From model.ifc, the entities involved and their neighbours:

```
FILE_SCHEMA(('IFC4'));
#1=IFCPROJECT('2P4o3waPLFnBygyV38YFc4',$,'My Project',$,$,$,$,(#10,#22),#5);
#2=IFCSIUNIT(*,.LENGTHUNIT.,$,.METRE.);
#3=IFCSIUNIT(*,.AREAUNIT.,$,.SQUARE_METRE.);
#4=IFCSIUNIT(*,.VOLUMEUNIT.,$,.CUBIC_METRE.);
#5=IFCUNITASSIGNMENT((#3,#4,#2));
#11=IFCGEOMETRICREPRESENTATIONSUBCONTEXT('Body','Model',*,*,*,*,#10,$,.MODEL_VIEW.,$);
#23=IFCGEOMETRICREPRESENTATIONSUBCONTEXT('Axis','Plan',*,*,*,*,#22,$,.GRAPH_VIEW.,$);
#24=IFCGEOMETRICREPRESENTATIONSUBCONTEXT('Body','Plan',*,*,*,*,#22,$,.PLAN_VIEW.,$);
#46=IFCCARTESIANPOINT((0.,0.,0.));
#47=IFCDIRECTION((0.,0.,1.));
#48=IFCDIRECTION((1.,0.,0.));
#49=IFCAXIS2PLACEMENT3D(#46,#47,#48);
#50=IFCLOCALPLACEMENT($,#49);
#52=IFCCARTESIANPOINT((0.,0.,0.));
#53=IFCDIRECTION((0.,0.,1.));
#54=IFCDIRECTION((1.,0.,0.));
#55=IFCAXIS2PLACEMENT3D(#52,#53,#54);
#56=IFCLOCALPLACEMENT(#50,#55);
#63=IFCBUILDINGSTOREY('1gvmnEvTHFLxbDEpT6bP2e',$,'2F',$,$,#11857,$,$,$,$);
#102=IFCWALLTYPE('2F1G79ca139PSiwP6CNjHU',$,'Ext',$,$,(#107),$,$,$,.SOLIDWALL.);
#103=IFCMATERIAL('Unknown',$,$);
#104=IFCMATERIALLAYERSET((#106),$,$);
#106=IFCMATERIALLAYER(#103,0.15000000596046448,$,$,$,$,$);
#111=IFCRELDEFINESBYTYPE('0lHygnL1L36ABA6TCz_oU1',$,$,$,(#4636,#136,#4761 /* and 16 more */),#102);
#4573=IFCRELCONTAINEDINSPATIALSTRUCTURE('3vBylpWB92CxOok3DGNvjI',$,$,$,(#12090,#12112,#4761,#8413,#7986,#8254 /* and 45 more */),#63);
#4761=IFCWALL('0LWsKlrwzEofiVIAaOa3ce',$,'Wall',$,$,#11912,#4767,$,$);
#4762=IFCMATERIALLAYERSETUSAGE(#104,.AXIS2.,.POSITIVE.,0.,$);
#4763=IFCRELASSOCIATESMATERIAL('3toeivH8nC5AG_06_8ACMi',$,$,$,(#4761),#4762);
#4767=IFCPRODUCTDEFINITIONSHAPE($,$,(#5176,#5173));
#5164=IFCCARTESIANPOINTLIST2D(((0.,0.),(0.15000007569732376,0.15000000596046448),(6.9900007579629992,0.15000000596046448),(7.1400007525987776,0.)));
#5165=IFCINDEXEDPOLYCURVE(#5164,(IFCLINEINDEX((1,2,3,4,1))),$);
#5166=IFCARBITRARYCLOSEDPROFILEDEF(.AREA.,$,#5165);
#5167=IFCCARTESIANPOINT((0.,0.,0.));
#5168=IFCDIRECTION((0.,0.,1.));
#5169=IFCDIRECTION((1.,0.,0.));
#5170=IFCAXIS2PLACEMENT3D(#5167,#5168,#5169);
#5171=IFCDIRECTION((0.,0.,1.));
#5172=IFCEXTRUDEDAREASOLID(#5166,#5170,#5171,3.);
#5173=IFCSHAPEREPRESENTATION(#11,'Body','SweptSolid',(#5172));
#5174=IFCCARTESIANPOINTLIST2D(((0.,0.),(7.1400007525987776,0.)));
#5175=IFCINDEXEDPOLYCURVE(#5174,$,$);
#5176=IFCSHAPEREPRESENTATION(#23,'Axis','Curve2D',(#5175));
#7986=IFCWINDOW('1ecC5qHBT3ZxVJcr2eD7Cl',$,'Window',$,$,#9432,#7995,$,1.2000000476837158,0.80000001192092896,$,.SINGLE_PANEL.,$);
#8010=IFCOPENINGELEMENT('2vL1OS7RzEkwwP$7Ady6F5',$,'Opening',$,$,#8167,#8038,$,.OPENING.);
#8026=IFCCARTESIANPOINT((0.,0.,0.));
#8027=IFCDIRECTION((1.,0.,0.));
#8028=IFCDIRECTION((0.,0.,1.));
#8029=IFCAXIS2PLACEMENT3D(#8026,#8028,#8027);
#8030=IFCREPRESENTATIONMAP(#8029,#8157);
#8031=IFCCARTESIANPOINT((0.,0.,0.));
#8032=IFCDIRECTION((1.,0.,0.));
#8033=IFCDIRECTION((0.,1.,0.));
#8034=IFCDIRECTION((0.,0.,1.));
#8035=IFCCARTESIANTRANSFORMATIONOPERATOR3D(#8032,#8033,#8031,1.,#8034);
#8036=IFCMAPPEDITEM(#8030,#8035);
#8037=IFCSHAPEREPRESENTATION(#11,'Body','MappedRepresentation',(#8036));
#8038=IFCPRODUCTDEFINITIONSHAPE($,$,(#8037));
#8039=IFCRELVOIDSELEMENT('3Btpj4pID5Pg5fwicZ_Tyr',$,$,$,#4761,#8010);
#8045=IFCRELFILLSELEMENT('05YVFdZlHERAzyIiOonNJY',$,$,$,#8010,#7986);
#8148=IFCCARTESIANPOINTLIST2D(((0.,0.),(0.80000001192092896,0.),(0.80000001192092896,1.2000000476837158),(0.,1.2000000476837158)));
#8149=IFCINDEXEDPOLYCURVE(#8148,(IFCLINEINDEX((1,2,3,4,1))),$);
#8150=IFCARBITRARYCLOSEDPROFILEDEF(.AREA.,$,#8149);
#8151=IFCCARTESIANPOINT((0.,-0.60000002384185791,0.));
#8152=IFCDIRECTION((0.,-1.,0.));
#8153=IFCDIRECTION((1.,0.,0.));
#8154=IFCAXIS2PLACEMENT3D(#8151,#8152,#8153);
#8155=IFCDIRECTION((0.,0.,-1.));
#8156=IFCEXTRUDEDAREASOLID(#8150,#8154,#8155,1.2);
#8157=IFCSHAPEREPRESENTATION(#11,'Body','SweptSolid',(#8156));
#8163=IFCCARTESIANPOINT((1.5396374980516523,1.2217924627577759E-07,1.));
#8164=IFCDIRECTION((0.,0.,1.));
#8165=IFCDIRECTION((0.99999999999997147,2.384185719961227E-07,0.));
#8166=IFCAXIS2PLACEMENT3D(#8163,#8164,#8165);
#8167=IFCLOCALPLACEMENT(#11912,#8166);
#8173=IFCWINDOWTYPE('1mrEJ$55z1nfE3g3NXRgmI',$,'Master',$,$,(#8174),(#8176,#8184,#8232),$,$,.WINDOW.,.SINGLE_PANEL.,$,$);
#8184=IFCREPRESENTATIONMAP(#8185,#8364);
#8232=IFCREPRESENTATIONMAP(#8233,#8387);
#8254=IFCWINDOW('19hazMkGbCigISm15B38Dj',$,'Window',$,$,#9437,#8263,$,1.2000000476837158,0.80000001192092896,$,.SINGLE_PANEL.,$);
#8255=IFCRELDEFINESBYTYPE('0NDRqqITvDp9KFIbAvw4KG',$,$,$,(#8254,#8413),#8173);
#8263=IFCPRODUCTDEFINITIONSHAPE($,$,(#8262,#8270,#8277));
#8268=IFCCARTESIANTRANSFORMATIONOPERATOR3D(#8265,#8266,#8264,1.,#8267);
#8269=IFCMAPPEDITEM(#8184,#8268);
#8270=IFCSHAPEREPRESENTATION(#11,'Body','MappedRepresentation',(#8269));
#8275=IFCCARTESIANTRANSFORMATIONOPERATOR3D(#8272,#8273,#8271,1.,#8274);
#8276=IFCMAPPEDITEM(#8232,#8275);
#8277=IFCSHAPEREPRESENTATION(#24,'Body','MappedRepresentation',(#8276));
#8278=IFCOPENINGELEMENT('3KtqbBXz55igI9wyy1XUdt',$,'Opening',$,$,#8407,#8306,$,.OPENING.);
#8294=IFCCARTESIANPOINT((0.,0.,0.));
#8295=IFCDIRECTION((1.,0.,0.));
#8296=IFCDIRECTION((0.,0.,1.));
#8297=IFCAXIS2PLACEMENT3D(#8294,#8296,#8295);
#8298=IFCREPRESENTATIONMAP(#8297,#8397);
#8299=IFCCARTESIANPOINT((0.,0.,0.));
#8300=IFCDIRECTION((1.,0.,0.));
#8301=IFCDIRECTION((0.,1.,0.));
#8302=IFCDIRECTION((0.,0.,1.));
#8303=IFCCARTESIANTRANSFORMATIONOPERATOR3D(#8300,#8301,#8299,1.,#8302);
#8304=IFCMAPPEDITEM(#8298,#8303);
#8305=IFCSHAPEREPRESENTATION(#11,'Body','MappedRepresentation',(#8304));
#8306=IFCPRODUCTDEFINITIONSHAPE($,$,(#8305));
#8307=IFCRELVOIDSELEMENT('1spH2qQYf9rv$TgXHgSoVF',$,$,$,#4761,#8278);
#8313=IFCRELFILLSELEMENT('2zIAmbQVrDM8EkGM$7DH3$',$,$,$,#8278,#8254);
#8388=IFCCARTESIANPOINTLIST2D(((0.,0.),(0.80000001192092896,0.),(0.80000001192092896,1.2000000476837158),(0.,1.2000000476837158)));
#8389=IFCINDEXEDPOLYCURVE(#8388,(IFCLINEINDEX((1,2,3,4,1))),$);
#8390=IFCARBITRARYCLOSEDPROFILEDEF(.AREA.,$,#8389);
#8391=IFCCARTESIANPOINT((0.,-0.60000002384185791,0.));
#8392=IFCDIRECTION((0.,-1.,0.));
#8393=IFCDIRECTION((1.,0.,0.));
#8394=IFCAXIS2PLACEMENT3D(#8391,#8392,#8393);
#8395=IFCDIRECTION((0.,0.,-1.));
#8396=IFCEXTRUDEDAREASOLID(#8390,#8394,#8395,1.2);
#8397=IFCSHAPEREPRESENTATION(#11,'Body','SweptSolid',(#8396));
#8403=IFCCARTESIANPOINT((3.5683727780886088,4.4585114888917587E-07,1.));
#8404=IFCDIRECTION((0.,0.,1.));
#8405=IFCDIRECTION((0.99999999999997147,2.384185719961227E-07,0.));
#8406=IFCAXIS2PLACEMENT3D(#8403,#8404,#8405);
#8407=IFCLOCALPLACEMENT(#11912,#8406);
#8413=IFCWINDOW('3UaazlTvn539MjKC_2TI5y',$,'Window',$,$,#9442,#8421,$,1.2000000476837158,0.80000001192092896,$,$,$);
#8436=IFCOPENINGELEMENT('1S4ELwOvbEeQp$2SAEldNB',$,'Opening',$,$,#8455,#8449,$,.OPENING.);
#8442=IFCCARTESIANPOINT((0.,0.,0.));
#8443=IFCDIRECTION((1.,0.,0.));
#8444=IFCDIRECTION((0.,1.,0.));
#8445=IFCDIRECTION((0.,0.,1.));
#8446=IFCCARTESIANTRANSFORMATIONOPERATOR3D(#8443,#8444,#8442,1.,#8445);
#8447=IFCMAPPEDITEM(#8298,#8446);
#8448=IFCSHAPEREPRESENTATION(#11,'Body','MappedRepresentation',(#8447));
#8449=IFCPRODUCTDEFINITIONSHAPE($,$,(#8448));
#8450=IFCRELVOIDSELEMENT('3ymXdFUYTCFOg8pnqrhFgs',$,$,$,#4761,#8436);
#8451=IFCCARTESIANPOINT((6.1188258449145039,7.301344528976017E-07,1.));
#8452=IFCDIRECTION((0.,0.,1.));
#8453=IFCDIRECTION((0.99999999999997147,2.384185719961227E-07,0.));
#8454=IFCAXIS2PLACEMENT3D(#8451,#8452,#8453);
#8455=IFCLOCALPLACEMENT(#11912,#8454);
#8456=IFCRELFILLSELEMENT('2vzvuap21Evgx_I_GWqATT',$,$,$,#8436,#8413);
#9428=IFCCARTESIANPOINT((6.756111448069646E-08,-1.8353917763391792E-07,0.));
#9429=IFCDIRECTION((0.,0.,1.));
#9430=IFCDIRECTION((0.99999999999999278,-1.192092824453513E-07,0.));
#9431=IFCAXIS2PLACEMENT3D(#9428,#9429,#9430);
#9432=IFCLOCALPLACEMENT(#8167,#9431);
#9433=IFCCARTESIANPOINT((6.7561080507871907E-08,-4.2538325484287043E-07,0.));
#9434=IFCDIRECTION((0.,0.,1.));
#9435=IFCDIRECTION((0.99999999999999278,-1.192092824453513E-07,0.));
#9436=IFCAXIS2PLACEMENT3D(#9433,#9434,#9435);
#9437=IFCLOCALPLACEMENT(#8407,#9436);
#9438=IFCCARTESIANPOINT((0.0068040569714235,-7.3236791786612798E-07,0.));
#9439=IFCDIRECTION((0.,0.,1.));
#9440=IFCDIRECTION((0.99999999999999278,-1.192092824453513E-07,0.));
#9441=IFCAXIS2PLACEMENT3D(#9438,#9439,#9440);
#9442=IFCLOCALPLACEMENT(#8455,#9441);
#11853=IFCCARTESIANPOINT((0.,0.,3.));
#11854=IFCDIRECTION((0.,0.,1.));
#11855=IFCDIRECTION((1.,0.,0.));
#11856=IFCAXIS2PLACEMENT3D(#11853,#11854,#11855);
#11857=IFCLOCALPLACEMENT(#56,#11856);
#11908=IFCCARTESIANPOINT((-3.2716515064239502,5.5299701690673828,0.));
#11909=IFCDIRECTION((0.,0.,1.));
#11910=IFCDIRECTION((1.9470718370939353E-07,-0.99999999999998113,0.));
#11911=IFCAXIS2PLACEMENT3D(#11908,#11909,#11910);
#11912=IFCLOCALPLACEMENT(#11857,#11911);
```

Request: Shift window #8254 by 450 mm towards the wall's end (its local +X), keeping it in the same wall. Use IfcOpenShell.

```python
import ifcopenshell
import ifcopenshell.api.geometry
import ifcopenshell.util.placement
import ifcopenshell.util.unit

model = ifcopenshell.open("model.ifc")
unit_scale = ifcopenshell.util.unit.calculate_unit_scale(model)

window = model.by_guid("19hazMkGbCigISm15B38Dj")
opening = window.FillsVoids[0].RelatingOpeningElement
wall = opening.VoidsElements[0].RelatingBuildingElement

wall_matrix = ifcopenshell.util.placement.get_local_placement(wall.ObjectPlacement)
shift = wall_matrix[:3, 0] * 0.45 / unit_scale
before = ifcopenshell.util.placement.get_local_placement(window.ObjectPlacement)[:3, 3].copy()

# The window is placed relative to its opening, so it follows when the opening moves.
matrix = ifcopenshell.util.placement.get_local_placement(opening.ObjectPlacement)
matrix[:3, 3] += shift
ifcopenshell.api.geometry.edit_object_placement(
    model, product=opening, matrix=matrix, is_si=False, should_transform_children=True
)

after = ifcopenshell.util.placement.get_local_placement(window.ObjectPlacement)[:3, 3]
print("window moved by", (after - before).round(3) + 0.0)

model.write("model_edited.ifc")
```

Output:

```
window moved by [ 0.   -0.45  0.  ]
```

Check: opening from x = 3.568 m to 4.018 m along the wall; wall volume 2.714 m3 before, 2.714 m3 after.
